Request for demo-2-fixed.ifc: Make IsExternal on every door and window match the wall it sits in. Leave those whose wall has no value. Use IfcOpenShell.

First a look at what the model holds.

```python
import ifcopenshell
import ifcopenshell.util.element

model = ifcopenshell.open("demo-2-fixed.ifc")
print(model.schema)
seen = {}
for e in model.by_type("IfcDoor") + model.by_type("IfcWindow"):
    if not e.FillsVoids:
        continue
    host = e.FillsVoids[0].RelatingOpeningElement.VoidsElements[0].RelatingBuildingElement
    own = ifcopenshell.util.element.get_pset(e, f"Pset_{e.is_a()[3:].removesuffix('StandardCase')}Common", "IsExternal")
    wall = ifcopenshell.util.element.get_pset(host, "Pset_WallCommon", "IsExternal")
    seen[e.is_a(), own, wall] = seen.get((e.is_a(), own, wall), 0) + 1
for (cls, own, wall), count in sorted(seen.items(), key=str):
    print(count, cls, "IsExternal:", own, "| host wall:", wall)
```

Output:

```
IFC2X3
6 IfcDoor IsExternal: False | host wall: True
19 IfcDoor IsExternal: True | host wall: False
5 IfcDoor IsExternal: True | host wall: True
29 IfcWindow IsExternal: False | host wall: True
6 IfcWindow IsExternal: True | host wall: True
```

```python
import ifcopenshell
import ifcopenshell.api.pset
import ifcopenshell.util.element

model = ifcopenshell.open("demo-2-fixed.ifc")

count = 0
for ifc_class, pset_name in (("IfcDoor", "Pset_DoorCommon"), ("IfcWindow", "Pset_WindowCommon")):
    for e in model.by_type(ifc_class):
        if not e.FillsVoids:
            continue
        host = e.FillsVoids[0].RelatingOpeningElement.VoidsElements[0].RelatingBuildingElement
        external = ifcopenshell.util.element.get_pset(host, "Pset_WallCommon", "IsExternal")
        if external is None or ifcopenshell.util.element.get_pset(e, pset_name, "IsExternal") == external:
            continue
        pset = ifcopenshell.api.pset.add_pset(model, product=e, name=pset_name)
        ifcopenshell.api.pset.edit_pset(model, pset=pset, properties={"IsExternal": external})
        count += 1

print(count, "updated")

model.write("demo-2-fixed_v2.ifc")
```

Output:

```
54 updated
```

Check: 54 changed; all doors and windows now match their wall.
